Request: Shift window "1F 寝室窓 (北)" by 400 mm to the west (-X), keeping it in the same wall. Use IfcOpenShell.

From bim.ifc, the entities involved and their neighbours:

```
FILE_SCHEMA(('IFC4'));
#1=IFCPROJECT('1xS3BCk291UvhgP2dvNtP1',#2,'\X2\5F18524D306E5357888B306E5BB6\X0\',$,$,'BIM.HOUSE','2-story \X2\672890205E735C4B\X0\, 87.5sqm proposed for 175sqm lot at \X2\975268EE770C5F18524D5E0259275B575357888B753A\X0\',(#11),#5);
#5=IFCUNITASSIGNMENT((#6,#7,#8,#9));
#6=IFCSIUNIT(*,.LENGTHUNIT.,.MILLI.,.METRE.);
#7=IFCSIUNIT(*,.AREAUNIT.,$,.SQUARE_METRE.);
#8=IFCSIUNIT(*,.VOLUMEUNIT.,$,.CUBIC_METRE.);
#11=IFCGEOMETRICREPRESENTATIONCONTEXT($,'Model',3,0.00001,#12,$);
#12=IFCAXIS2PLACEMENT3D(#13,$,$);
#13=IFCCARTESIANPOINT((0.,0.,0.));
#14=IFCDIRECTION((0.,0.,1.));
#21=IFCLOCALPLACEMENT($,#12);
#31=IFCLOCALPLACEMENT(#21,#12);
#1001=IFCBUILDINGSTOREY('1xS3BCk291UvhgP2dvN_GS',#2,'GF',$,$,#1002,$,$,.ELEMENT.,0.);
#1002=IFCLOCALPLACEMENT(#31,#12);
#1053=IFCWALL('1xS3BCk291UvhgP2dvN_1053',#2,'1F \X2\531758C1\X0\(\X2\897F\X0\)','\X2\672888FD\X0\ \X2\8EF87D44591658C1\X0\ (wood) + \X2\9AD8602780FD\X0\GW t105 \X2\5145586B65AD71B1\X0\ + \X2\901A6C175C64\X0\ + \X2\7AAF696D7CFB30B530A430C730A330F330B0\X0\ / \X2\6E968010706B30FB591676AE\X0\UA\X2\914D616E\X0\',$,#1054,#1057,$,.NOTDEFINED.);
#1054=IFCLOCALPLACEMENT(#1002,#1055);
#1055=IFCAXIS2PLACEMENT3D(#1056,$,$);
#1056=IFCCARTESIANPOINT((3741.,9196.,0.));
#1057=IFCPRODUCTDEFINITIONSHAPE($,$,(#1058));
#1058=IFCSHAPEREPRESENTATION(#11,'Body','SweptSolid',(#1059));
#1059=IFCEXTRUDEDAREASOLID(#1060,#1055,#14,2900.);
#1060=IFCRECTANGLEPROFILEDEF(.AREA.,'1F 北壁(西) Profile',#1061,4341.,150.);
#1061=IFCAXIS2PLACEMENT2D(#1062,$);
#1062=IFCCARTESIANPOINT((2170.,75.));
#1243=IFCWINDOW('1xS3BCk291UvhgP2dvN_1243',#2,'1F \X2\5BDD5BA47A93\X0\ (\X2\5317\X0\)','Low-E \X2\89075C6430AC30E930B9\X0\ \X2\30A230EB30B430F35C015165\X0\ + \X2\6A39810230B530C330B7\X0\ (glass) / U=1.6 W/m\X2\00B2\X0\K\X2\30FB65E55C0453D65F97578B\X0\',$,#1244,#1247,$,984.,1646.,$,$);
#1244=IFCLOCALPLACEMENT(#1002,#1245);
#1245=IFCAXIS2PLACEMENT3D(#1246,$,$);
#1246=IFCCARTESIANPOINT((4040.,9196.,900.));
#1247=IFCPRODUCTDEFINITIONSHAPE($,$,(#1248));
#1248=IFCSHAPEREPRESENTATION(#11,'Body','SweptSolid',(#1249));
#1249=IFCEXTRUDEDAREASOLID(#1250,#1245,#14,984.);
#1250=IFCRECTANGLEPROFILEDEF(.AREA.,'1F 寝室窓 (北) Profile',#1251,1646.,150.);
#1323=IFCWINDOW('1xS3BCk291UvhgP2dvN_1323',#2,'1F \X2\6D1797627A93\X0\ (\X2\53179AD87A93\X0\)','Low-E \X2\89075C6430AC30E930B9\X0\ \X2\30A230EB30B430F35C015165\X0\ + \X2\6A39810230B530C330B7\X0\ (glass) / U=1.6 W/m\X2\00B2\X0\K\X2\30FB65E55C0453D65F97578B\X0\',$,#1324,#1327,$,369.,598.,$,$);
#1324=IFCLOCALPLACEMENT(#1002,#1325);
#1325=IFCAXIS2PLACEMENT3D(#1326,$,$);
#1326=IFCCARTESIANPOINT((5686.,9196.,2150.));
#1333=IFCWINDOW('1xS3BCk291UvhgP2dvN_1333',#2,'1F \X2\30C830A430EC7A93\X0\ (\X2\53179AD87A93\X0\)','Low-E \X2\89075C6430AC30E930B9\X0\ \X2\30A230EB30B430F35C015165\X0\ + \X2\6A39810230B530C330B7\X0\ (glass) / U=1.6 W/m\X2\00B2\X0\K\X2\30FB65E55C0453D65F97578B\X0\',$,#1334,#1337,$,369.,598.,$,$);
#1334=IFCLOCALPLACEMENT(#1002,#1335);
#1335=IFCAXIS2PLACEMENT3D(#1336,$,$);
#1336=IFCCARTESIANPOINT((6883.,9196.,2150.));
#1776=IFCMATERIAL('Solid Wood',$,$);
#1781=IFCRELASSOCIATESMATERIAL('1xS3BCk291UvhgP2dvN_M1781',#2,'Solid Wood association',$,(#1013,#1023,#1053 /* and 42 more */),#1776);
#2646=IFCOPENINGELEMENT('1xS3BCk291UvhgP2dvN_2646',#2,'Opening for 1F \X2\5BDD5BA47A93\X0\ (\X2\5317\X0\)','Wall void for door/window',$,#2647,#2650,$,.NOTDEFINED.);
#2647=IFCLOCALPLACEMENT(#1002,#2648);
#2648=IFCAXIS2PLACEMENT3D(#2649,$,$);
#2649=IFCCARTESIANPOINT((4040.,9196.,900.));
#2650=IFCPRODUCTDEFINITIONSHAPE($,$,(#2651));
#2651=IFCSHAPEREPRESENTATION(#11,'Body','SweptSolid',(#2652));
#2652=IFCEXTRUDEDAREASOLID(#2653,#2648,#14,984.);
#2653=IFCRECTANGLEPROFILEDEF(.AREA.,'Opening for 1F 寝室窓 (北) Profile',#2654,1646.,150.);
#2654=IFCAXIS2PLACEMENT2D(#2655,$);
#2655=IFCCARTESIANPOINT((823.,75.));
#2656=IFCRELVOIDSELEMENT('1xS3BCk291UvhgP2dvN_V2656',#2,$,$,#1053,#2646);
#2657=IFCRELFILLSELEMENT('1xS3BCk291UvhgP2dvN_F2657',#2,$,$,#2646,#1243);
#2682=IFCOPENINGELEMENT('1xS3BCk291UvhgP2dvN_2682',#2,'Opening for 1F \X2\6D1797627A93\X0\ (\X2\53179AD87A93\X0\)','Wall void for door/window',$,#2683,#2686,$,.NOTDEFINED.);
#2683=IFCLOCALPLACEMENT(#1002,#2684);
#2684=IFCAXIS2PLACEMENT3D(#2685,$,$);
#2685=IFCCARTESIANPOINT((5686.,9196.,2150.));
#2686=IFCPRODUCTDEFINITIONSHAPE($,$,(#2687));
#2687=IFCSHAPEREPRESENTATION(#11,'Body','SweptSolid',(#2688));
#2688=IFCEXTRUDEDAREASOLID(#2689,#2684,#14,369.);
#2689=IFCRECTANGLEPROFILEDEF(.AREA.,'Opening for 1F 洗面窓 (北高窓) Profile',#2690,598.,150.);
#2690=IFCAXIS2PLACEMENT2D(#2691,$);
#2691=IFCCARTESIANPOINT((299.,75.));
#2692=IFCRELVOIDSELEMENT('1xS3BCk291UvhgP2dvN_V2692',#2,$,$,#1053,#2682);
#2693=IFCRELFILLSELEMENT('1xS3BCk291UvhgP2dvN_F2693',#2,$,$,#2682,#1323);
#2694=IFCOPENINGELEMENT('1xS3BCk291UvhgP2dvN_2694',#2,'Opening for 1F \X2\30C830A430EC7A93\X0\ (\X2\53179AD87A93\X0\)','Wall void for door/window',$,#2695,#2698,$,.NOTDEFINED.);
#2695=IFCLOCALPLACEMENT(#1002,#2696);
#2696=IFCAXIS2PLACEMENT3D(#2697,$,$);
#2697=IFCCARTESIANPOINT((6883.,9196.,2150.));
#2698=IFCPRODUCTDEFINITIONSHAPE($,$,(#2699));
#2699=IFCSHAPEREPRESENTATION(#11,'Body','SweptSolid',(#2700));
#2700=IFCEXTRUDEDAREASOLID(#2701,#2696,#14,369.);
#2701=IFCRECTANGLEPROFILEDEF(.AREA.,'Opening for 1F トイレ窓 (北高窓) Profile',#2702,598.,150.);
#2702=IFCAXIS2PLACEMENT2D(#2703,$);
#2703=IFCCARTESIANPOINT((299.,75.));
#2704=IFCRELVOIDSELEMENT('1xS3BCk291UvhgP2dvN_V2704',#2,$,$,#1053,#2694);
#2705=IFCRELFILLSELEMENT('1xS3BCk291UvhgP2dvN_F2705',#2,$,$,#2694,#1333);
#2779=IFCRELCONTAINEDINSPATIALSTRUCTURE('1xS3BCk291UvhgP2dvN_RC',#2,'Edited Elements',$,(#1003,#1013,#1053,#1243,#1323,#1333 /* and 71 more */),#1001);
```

```python
import ifcopenshell
import ifcopenshell.api.geometry
import ifcopenshell.util.placement

model = ifcopenshell.open("bim.ifc")

window = model.by_id(1243)
opening = window.FillsVoids[0].RelatingOpeningElement
wall = opening.VoidsElements[0].RelatingBuildingElement

wall_matrix = ifcopenshell.util.placement.get_local_placement(wall.ObjectPlacement)
shift = wall_matrix[:3, 0] * -400.0
before = ifcopenshell.util.placement.get_local_placement(window.ObjectPlacement)[:3, 3].copy()

# The window is not placed relative to its opening, so move both.
for product in (opening, window):
    matrix = ifcopenshell.util.placement.get_local_placement(product.ObjectPlacement)
    matrix[:3, 3] += shift
    ifcopenshell.api.geometry.edit_object_placement(model, product=product, matrix=matrix, is_si=False)

after = ifcopenshell.util.placement.get_local_placement(window.ObjectPlacement)[:3, 3]
print("window moved by", (after - before).round(3) + 0.0)

model.write("bim-out.ifc")
```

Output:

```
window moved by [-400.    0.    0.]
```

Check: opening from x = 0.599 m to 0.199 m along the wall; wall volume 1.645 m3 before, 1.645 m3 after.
